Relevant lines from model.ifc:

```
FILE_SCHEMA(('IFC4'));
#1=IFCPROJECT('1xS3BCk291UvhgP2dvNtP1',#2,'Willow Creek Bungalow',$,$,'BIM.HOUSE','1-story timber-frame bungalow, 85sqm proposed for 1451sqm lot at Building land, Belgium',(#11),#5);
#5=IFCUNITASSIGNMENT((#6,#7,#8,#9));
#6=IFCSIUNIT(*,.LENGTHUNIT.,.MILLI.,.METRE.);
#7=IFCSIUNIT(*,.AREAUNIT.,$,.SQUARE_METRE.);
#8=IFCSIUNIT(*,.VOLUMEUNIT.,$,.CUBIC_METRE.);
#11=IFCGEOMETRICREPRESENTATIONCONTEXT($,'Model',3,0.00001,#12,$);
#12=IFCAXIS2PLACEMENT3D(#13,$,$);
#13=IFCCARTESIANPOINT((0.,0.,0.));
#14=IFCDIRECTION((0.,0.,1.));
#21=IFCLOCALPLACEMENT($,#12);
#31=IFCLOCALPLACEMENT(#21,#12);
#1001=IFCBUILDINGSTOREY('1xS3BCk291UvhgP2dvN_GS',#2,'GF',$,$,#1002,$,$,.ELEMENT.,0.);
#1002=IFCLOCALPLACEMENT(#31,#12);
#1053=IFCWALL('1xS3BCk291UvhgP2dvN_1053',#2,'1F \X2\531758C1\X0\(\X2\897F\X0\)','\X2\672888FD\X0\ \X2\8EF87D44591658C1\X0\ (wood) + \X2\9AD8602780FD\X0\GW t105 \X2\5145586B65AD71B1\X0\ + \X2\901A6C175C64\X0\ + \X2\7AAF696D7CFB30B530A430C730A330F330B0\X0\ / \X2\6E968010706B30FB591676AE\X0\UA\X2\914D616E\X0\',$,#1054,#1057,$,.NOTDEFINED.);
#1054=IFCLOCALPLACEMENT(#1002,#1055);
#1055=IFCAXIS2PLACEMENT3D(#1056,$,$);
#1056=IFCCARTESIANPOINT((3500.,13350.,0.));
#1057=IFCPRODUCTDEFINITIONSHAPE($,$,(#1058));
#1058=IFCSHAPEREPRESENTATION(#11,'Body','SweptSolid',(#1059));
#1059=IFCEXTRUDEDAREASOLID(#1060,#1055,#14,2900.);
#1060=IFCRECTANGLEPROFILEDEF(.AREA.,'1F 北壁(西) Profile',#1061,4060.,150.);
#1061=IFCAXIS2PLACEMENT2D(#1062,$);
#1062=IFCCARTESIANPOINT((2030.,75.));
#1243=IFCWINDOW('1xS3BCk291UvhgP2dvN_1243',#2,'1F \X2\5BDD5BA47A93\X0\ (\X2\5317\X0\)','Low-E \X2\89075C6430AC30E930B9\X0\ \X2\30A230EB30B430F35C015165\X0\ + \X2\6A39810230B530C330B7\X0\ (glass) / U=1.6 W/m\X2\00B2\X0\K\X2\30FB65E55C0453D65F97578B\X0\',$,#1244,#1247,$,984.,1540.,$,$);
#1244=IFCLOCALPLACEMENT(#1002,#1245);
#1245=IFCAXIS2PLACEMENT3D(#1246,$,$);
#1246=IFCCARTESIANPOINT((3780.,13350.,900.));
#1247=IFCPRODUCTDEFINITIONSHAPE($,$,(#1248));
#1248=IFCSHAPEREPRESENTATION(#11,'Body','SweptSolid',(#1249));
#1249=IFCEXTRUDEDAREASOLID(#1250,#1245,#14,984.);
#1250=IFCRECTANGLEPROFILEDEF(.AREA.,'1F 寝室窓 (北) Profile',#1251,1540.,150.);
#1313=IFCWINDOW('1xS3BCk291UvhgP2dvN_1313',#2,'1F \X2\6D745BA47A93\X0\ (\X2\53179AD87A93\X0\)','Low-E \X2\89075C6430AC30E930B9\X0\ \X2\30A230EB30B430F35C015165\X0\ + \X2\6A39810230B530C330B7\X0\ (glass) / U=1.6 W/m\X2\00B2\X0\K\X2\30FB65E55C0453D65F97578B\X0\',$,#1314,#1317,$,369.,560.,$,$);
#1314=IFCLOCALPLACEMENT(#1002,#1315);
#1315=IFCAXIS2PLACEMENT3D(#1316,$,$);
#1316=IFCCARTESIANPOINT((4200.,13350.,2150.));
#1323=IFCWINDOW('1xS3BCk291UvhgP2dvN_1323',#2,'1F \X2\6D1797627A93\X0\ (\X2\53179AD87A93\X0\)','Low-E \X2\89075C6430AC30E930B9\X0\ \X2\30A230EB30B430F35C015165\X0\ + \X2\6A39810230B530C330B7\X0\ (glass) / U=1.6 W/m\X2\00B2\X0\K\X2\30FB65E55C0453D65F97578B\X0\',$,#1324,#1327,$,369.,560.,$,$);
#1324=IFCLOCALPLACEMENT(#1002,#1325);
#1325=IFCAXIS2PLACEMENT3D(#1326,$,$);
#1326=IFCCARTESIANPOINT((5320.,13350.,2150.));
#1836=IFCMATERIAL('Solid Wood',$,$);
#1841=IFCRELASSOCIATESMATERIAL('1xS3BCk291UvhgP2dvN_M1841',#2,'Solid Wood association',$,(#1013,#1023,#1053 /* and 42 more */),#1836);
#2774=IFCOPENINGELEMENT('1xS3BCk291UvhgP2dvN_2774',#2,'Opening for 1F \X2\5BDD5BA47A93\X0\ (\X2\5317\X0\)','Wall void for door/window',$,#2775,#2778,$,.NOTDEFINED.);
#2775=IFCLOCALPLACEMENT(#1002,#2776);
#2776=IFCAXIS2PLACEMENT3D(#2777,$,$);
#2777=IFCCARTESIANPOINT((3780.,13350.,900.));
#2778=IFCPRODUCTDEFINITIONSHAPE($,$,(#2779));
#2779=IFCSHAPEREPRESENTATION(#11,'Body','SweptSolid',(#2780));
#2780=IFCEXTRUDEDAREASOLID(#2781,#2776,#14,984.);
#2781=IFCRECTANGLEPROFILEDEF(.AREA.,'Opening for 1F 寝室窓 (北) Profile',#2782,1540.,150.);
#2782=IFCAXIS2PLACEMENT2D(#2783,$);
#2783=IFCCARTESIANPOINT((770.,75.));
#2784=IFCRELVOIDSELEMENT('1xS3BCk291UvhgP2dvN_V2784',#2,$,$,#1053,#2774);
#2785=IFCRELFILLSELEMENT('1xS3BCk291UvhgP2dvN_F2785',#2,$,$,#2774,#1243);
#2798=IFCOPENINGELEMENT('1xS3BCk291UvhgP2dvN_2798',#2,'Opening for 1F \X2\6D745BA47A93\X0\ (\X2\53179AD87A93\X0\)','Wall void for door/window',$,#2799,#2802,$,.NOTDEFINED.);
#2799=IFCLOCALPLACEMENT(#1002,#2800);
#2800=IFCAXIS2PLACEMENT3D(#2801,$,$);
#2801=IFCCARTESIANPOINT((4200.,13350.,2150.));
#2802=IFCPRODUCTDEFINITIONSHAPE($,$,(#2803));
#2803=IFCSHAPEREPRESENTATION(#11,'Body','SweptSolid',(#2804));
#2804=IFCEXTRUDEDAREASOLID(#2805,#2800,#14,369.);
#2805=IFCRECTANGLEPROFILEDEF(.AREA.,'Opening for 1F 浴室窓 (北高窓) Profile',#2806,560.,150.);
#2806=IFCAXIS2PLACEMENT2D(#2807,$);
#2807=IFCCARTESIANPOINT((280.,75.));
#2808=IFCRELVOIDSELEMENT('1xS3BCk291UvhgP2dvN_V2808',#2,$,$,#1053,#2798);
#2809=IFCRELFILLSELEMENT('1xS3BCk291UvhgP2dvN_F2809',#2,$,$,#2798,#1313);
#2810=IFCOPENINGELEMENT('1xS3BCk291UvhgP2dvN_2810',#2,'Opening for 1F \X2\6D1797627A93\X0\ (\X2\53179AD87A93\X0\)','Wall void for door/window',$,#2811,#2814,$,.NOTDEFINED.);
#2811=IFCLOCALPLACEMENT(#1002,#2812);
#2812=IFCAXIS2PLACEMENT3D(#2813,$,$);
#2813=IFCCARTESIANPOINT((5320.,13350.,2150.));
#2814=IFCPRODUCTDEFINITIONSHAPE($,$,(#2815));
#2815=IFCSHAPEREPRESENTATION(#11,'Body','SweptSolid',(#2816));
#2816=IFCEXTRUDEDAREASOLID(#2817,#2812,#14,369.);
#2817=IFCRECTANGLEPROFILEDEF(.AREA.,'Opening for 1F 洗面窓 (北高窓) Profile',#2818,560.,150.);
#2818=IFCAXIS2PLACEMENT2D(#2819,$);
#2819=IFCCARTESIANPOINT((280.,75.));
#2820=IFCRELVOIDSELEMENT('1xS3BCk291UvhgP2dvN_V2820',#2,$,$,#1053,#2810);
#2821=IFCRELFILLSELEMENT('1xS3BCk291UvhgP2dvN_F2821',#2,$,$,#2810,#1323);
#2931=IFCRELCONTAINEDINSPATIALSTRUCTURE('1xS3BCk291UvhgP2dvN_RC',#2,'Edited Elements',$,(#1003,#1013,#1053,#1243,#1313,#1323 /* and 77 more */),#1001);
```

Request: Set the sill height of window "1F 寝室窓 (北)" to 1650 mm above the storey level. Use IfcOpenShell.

```python
import numpy as np
import ifcopenshell
import ifcopenshell.api.geometry
import ifcopenshell.geom
import ifcopenshell.util.element
import ifcopenshell.util.placement
import ifcopenshell.util.shape
import ifcopenshell.util.unit

model = ifcopenshell.open("model.ifc")
unit_scale = ifcopenshell.util.unit.calculate_unit_scale(model)

window = model.by_guid("1xS3BCk291UvhgP2dvN_1243")
opening = window.FillsVoids[0].RelatingOpeningElement
storey = ifcopenshell.util.element.get_container(window, ifc_class="IfcBuildingStorey")
level = ifcopenshell.util.placement.get_local_placement(storey.ObjectPlacement)[2, 3]

# The opening's origin need not be at the sill, so measure its lowest point.
shape = ifcopenshell.geom.create_shape(ifcopenshell.geom.settings(), opening)
bottom = ifcopenshell.util.shape.get_shape_bottom_elevation(shape, shape.geometry) / unit_scale
dz = level + 1650.0 - bottom

shift = np.array([0.0, 0.0, dz])
# The window is not placed relative to its opening, so move both.
for product in (opening, window):
    matrix = ifcopenshell.util.placement.get_local_placement(product.ObjectPlacement)
    matrix[:3, 3] += shift
    ifcopenshell.api.geometry.edit_object_placement(model, product=product, matrix=matrix, is_si=False)

print(f"moved by {dz * unit_scale:+.3f} m")

model.write("model-out.ifc")
```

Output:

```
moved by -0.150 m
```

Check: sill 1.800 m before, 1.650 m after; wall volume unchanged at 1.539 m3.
